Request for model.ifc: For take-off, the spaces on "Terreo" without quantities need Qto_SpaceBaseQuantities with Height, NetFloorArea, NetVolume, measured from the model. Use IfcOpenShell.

First a look at what the model holds.

```python
import ifcopenshell
import ifcopenshell.util.element
import ifcopenshell.util.unit

model = ifcopenshell.open("model.ifc")
print(model.schema)
for unit_type in ("LENGTHUNIT", "AREAUNIT", "VOLUMEUNIT"):
    print(unit_type, ifcopenshell.util.unit.calculate_unit_scale(model, unit_type))
storey = next(s for s in model.by_type("IfcBuildingStorey") if s.Name == "Terreo")
spaces = [e for e in ifcopenshell.util.element.get_decomposition(storey) if e.is_a("IfcSpace")]
for e in sorted(spaces, key=lambda e: e.id()):
    print(e.id(), e.is_a(), e.Name, list(ifcopenshell.util.element.get_psets(e, qtos_only=True)), sep=" | ")
```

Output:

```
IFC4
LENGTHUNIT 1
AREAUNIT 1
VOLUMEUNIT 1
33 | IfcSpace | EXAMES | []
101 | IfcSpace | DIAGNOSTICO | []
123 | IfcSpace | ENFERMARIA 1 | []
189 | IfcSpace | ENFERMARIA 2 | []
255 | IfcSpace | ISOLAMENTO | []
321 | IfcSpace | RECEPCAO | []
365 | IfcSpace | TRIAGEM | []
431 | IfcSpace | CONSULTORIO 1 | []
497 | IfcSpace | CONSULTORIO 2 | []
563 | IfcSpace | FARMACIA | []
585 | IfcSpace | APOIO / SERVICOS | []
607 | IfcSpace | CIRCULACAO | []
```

```python
import ifcopenshell
import ifcopenshell.api.pset
import ifcopenshell.geom
import ifcopenshell.util.element
import ifcopenshell.util.shape
import ifcopenshell.util.unit

model = ifcopenshell.open("model.ifc")
unit_scale = ifcopenshell.util.unit.calculate_unit_scale(model)
area_scale = ifcopenshell.util.unit.calculate_unit_scale(model, "AREAUNIT")
volume_scale = ifcopenshell.util.unit.calculate_unit_scale(model, "VOLUMEUNIT")
settings = ifcopenshell.geom.settings()

storey = next(s for s in model.by_type("IfcBuildingStorey") if s.Name == "Terreo")
spaces = [e for e in ifcopenshell.util.element.get_decomposition(storey) if e.is_a("IfcSpace")]

for e in sorted(spaces, key=lambda e: e.id()):
    if ifcopenshell.util.element.get_psets(e, qtos_only=True, should_inherit=False):
        continue
    # Geometry comes back in metres, in the element's own axes.
    shape = ifcopenshell.geom.create_shape(settings, e)
    values = {
        "Height": ifcopenshell.util.shape.get_z(shape.geometry) / unit_scale,
        "NetFloorArea": ifcopenshell.util.shape.get_footprint_area(shape.geometry) / area_scale,
        "NetVolume": ifcopenshell.util.shape.get_volume(shape.geometry) / volume_scale,
    }
    qto = ifcopenshell.api.pset.add_qto(model, product=e, name="Qto_SpaceBaseQuantities")
    ifcopenshell.api.pset.edit_qto(model, qto=qto, properties=values)
    print(e.id(), {k: round(v, 3) for k, v in values.items()})

model.write("model_updated.ifc")
```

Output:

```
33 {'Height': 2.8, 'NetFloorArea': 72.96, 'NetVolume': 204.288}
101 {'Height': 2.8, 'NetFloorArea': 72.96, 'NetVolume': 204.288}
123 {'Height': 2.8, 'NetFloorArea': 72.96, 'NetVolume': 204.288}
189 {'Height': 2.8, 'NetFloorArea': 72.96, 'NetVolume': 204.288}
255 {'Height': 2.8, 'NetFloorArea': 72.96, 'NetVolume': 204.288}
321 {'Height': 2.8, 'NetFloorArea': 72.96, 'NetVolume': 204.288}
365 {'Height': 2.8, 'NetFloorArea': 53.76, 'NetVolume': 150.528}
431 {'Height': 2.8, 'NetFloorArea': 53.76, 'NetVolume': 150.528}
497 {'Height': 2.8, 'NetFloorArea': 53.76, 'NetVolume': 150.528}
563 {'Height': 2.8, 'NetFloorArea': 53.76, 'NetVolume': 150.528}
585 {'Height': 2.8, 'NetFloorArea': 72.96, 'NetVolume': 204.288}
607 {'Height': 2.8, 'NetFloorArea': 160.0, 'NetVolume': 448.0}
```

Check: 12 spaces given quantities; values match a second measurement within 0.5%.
